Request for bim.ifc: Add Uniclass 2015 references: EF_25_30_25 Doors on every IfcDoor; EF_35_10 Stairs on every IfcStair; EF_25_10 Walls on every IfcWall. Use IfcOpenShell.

First a look at what the model holds.

```python
import ifcopenshell

model = ifcopenshell.open("bim.ifc")
print(model.schema)
print("classifications:", [c.Name for c in model.by_type("IfcClassification")])
for ifc_class in ("IfcDoor", "IfcRoof", "IfcStair", "IfcWall", "IfcWindow"):
    print(ifc_class, len(model.by_type(ifc_class)))
```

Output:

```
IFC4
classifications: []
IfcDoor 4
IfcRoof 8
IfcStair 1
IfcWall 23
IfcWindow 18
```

```python
import ifcopenshell
import ifcopenshell.api.classification

model = ifcopenshell.open("bim.ifc")

system = ifcopenshell.api.classification.add_classification(model, classification="Uniclass 2015")

codes = {
    "IfcDoor": ("EF_25_30_25", "Doors"),
    "IfcStair": ("EF_35_10", "Stairs"),
    "IfcWall": ("EF_25_10", "Walls"),
}
for ifc_class, (code, name) in codes.items():
    products = model.by_type(ifc_class)
    ifcopenshell.api.classification.add_reference(
        model, products=products, classification=system, identification=code, name=name
    )
    print(code, len(products))

model.write("bim_updated.ifc")
```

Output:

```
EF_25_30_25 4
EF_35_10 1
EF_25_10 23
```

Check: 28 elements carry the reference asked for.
